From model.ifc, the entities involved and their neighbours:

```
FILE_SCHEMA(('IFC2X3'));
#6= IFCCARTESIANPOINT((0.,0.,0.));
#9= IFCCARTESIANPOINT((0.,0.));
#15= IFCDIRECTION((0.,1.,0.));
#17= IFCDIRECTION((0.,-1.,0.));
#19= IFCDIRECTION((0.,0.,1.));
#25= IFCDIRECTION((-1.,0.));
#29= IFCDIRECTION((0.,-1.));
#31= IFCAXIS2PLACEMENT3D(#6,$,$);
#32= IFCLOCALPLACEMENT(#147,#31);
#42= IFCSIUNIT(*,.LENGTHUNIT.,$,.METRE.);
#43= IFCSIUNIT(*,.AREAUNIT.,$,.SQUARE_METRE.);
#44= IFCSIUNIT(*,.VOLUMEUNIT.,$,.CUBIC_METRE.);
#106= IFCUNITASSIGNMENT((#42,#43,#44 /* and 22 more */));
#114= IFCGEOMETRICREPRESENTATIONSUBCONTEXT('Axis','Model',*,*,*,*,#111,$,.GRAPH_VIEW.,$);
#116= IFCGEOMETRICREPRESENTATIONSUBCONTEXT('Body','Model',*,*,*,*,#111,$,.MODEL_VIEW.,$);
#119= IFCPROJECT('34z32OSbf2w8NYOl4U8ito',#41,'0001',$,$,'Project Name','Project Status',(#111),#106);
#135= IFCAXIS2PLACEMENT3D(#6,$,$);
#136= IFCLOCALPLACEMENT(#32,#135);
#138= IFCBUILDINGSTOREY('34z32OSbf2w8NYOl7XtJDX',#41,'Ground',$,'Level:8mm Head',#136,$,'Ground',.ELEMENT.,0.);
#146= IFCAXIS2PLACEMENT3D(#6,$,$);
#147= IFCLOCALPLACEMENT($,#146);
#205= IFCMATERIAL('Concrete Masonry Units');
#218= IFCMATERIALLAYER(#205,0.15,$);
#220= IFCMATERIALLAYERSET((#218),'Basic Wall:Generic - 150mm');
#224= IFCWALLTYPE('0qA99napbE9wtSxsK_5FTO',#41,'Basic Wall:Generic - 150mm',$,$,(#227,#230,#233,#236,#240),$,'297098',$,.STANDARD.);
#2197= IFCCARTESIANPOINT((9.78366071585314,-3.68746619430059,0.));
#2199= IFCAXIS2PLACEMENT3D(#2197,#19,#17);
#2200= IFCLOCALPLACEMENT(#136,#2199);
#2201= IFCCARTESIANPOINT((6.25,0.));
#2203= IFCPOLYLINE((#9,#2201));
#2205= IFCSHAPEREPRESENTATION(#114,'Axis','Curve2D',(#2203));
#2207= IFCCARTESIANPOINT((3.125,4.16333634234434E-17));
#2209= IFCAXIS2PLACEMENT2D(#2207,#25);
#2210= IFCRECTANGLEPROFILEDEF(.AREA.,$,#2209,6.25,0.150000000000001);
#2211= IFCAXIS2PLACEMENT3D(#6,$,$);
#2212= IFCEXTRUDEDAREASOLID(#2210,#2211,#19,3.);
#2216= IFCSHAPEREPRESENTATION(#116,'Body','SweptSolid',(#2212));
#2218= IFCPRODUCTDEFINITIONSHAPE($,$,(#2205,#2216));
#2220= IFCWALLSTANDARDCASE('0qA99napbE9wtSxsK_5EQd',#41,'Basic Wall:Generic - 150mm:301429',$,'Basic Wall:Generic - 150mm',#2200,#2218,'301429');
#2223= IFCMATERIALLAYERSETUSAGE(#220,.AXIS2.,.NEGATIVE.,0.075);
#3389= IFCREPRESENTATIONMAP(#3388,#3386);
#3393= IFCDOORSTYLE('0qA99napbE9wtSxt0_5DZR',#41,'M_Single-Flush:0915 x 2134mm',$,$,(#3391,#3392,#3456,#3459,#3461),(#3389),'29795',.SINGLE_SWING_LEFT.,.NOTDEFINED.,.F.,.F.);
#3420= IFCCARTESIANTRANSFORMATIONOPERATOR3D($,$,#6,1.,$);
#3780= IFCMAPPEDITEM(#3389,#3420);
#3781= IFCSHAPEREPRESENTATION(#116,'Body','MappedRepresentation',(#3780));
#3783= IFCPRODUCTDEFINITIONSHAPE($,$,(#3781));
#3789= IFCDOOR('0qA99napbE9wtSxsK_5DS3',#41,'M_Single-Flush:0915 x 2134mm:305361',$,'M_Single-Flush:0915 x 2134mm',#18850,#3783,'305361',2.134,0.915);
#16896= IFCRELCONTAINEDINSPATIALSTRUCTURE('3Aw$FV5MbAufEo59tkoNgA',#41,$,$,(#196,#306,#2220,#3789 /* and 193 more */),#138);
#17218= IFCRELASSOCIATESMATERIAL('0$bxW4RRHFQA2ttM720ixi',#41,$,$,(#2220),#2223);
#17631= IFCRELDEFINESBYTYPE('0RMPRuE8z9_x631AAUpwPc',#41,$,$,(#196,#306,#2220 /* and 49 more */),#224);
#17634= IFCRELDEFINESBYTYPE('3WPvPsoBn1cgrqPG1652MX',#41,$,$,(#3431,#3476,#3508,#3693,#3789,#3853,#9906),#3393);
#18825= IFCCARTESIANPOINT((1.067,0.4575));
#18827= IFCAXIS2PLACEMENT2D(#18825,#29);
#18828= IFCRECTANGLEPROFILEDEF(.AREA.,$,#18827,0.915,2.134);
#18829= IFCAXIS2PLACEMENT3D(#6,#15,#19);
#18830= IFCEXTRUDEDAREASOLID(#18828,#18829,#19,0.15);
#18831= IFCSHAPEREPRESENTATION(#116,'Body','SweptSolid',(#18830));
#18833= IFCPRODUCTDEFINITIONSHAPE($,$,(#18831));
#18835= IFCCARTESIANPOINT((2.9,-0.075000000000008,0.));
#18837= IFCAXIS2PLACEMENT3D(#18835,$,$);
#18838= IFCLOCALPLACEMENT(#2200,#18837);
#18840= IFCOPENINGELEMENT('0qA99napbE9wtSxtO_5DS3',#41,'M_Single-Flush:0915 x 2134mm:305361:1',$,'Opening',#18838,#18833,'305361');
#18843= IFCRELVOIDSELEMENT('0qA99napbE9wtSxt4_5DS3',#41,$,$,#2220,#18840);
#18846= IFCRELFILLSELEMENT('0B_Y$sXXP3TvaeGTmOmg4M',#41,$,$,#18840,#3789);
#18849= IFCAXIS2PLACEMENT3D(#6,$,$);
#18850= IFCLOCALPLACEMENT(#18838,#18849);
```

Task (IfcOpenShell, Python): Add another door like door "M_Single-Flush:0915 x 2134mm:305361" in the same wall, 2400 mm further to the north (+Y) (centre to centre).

```python
import ifcopenshell
import ifcopenshell.api.feature
import ifcopenshell.api.geometry
import ifcopenshell.api.root
import ifcopenshell.geom
import ifcopenshell.util.element
import ifcopenshell.util.placement
import ifcopenshell.util.shape
import ifcopenshell.util.unit

model = ifcopenshell.open("model.ifc")
unit_scale = ifcopenshell.util.unit.calculate_unit_scale(model)
settings = ifcopenshell.geom.settings()


def volume(element):
    """Net volume in cubic metres, openings subtracted."""
    shape = ifcopenshell.geom.create_shape(settings, element)
    return ifcopenshell.util.shape.get_volume(shape.geometry)


def reuse_history(source, copy):
    """copy_class also copies each property set's owner history, people and application; keep the originals."""
    for rel in copy.IsDefinedBy:
        if rel.is_a("IfcRelDefinesByProperties") and (history := rel.RelatingPropertyDefinition.OwnerHistory):
            rel.RelatingPropertyDefinition.OwnerHistory = source.OwnerHistory
            ifcopenshell.util.element.remove_deep2(model, history)


door = model.by_id(3789)
opening = door.FillsVoids[0].RelatingOpeningElement
wall = opening.VoidsElements[0].RelatingBuildingElement
before = volume(wall)
shift = ifcopenshell.util.placement.get_local_placement(wall.ObjectPlacement)[:3, 0] * -2.4 / unit_scale

# copy_class copies the void relationship, type, container and properties, but no geometry.
new_opening = ifcopenshell.api.root.copy_class(model, product=opening)
new_opening.Representation = ifcopenshell.util.element.copy_deep(
    model, opening.Representation, exclude=["IfcGeometricRepresentationContext", "IfcRepresentationMap"]
)
new_opening.Name = "M_Single-Flush:0915 x 2134mm"
new_opening.Tag = None
new_door = ifcopenshell.api.root.copy_class(model, product=door)
new_door.Representation = ifcopenshell.util.element.copy_deep(
    model, door.Representation, exclude=["IfcGeometricRepresentationContext", "IfcRepresentationMap"]
)
new_door.Name = "M_Single-Flush:0915 x 2134mm"
new_door.Tag = None
reuse_history(door, new_door)
fills = ifcopenshell.api.feature.add_filling(model, opening=new_opening, element=new_door)
fills.OwnerHistory = new_door.OwnerHistory  # required in IFC2X3

for old, new in ((opening, new_opening), (door, new_door)):
    matrix = ifcopenshell.util.placement.get_local_placement(old.ObjectPlacement)
    matrix[:3, 3] += shift
    ifcopenshell.api.geometry.edit_object_placement(model, product=new, matrix=matrix, is_si=False)

after = volume(wall)

print(f"wall volume {before:.3f} -> {after:.3f} m3")

model.write("model_edited.ifc")
```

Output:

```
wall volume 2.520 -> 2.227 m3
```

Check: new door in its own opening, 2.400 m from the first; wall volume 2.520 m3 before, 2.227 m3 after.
